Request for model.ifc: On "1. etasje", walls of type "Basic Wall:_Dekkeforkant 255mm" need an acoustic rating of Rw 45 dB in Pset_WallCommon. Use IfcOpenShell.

First a look at what the model holds.

```python
import ifcopenshell
import ifcopenshell.util.element

model = ifcopenshell.open("model.ifc")
print(model.schema)
storey = next(s for s in model.by_type("IfcBuildingStorey") if s.Name == "1. etasje")
walls = [e for e in ifcopenshell.util.element.get_decomposition(storey) if e.is_a("IfcWall")]
seen = {}
for e in walls:
    element_type = ifcopenshell.util.element.get_type(e)
    key = (element_type.Name if element_type != e and element_type else None, ifcopenshell.util.element.get_pset(e, "Pset_WallCommon", "AcousticRating"))
    seen[key] = seen.get(key, 0) + 1
for (name, value), count in sorted(seen.items(), key=str):
    print(count, "x", name, "|", value)
```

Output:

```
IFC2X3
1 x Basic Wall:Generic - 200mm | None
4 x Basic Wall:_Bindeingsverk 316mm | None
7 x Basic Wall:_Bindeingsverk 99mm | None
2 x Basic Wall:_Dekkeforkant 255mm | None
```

```python
import ifcopenshell
import ifcopenshell.api.pset
import ifcopenshell.util.element

model = ifcopenshell.open("model.ifc")

storey = next(s for s in model.by_type("IfcBuildingStorey") if s.Name == "1. etasje")
walls = [e for e in ifcopenshell.util.element.get_decomposition(storey) if e.is_a("IfcWall")]

count = 0
for e in walls:
    element_type = ifcopenshell.util.element.get_type(e)
    if element_type in (None, e) or element_type.Name != "Basic Wall:_Dekkeforkant 255mm":
        continue
    # add_pset returns the element's existing set when there is one.
    pset = ifcopenshell.api.pset.add_pset(model, product=e, name="Pset_WallCommon")
    ifcopenshell.api.pset.edit_pset(model, pset=pset, properties={"AcousticRating": "Rw 45 dB"})
    count += 1

print(count, "walls updated")

model.write("model_v2.ifc")
```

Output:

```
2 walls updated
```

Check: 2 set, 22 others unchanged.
